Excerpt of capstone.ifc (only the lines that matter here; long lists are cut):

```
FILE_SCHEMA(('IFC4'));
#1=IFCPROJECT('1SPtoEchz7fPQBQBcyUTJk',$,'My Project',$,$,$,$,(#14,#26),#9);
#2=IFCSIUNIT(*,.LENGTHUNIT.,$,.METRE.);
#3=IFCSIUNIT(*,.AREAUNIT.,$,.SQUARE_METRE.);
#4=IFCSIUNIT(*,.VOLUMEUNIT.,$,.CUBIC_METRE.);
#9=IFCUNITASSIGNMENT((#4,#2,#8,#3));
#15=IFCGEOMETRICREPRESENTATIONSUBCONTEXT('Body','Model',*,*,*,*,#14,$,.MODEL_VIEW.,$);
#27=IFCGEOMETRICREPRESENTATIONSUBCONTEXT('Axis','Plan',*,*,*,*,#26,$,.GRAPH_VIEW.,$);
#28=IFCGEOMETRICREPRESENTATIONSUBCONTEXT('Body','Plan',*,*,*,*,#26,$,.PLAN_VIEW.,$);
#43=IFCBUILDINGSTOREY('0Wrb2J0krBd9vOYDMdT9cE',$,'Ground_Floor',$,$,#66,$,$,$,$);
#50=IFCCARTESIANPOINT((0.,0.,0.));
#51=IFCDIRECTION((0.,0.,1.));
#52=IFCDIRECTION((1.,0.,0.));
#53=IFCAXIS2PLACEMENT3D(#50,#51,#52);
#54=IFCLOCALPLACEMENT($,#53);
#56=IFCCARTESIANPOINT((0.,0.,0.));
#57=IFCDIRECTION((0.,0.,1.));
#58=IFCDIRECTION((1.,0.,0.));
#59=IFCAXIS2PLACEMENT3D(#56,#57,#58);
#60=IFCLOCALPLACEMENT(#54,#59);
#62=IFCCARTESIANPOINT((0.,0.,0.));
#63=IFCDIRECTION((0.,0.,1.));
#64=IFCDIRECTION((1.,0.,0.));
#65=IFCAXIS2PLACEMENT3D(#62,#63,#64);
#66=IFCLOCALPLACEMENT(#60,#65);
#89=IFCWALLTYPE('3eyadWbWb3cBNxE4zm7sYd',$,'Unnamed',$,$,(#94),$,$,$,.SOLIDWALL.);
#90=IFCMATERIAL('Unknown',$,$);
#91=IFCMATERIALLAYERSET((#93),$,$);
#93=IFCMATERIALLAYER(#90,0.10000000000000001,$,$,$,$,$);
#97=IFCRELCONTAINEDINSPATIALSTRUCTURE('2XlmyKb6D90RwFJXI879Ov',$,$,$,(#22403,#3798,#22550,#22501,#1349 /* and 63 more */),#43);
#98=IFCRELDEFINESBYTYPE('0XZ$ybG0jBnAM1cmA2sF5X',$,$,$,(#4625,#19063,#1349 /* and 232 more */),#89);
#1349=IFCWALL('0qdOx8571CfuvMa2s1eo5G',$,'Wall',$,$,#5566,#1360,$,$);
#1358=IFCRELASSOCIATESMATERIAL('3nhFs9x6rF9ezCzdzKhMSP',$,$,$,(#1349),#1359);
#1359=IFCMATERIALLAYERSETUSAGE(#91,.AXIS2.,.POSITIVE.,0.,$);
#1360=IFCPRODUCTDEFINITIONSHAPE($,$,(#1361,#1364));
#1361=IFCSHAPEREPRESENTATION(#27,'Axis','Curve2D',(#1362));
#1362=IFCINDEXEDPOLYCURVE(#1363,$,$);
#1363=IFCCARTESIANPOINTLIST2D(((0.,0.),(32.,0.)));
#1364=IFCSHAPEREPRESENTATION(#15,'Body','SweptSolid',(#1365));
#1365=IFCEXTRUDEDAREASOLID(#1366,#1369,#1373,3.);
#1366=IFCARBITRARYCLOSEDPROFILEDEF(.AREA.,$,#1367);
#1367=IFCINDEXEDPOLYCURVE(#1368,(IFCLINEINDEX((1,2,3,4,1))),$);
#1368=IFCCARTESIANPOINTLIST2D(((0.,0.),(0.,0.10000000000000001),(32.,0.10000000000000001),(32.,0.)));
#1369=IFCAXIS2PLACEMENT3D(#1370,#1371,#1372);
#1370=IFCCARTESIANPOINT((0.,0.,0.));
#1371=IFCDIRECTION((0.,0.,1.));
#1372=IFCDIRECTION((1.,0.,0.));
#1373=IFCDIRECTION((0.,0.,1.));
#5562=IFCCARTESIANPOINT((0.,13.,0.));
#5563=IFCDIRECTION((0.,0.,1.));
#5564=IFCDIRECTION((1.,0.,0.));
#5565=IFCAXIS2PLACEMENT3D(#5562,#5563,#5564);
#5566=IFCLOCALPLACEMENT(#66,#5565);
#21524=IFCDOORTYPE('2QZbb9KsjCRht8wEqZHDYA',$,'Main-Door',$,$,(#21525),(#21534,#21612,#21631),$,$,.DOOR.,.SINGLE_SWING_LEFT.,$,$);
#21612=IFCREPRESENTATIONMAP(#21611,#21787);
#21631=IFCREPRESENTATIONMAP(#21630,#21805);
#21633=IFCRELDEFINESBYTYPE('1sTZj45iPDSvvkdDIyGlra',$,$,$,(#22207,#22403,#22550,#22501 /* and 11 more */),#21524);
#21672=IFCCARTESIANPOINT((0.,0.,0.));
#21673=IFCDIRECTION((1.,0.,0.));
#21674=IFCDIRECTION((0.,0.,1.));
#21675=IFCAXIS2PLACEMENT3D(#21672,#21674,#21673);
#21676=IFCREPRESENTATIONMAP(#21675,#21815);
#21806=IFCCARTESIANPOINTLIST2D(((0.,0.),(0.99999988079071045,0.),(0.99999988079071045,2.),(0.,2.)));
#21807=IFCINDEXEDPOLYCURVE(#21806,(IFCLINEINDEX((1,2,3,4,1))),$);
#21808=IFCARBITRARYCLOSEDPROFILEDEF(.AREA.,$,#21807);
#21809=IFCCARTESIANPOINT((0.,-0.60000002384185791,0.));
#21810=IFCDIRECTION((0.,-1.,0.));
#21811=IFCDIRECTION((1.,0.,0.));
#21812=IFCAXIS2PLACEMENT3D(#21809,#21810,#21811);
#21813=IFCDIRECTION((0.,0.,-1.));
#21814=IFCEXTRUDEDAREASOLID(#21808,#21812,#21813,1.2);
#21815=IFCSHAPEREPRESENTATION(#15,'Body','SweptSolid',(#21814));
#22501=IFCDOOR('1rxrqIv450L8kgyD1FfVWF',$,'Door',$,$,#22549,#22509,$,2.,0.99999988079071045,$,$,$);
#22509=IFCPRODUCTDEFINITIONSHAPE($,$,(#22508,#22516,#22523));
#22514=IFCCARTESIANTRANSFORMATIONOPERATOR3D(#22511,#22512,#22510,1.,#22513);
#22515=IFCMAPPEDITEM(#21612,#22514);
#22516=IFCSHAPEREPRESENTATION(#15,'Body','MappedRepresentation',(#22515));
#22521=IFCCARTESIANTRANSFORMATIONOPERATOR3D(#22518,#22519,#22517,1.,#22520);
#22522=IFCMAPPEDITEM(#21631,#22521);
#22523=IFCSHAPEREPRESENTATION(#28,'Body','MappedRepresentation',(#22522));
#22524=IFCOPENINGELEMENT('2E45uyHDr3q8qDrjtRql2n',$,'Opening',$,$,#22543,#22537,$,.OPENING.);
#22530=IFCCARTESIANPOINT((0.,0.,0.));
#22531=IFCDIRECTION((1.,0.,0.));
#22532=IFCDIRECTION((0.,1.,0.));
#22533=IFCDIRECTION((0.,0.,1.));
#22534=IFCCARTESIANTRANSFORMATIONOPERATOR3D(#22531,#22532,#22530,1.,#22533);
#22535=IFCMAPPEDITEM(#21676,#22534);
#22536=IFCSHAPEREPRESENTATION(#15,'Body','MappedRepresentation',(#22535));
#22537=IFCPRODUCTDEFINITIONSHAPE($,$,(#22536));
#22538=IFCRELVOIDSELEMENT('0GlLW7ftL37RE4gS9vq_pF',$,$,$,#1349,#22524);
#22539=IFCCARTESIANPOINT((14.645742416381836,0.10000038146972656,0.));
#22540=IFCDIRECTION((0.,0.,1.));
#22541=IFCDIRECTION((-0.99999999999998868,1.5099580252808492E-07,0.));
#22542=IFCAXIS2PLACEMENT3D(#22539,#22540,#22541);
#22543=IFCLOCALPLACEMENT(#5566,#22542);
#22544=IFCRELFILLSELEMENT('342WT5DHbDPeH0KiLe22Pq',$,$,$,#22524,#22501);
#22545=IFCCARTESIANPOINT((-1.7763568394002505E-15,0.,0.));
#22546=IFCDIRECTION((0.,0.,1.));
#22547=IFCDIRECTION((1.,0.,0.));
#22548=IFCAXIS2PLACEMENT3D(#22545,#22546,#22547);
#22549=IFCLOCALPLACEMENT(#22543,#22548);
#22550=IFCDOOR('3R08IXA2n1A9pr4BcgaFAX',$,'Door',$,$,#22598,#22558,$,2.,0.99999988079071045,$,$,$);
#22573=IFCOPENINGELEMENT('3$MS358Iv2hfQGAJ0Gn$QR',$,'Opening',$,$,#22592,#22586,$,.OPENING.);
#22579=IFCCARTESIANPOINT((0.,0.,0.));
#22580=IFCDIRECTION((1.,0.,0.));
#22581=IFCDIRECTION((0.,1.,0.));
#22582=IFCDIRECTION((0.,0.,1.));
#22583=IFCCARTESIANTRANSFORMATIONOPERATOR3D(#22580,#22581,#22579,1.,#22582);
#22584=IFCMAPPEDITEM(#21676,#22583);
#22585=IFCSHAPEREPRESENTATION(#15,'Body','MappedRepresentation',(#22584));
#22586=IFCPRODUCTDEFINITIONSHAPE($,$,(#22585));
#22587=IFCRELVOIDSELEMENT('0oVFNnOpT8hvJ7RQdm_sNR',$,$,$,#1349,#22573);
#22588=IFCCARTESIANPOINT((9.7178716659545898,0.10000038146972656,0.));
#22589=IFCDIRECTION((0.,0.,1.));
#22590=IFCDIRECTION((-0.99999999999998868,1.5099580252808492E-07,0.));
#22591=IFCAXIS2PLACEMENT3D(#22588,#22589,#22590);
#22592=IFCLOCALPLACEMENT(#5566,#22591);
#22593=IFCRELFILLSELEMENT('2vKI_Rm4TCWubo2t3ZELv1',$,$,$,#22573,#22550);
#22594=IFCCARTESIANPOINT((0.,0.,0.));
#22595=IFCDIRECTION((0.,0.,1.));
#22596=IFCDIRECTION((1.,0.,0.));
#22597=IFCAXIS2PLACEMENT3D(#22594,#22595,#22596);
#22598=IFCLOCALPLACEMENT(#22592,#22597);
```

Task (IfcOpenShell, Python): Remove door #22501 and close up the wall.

```python
import ifcopenshell
import ifcopenshell.api.feature
import ifcopenshell.api.root
import ifcopenshell.geom
import ifcopenshell.util.shape

model = ifcopenshell.open("capstone.ifc")
settings = ifcopenshell.geom.settings()


def volume(element):
    """Net volume in cubic metres, openings subtracted."""
    shape = ifcopenshell.geom.create_shape(settings, element)
    return ifcopenshell.util.shape.get_volume(shape.geometry)


door = model.by_guid("1rxrqIv450L8kgyD1FfVWF")
opening = door.FillsVoids[0].RelatingOpeningElement
wall = opening.VoidsElements[0].RelatingBuildingElement
before = volume(wall)

ifcopenshell.api.root.remove_product(model, product=door)
ifcopenshell.api.feature.remove_feature(model, feature=opening)

after = volume(wall)

print(f"wall volume {before:.3f} -> {after:.3f} m3")

model.write("capstone_rev.ifc")
```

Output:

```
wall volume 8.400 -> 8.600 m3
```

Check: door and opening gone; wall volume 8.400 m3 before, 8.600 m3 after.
